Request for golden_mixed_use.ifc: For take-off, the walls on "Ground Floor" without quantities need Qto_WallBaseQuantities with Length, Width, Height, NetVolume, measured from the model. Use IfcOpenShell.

First a look at what the model holds.

```python
import ifcopenshell
import ifcopenshell.util.element
import ifcopenshell.util.unit

model = ifcopenshell.open("golden_mixed_use.ifc")
print(model.schema)
for unit_type in ("LENGTHUNIT", "AREAUNIT", "VOLUMEUNIT"):
    print(unit_type, ifcopenshell.util.unit.calculate_unit_scale(model, unit_type))
storey = next(s for s in model.by_type("IfcBuildingStorey") if s.Name == "Ground Floor")
walls = [e for e in ifcopenshell.util.element.get_decomposition(storey) if e.is_a("IfcWall")]
for e in sorted(walls, key=lambda e: e.id()):
    print(e.id(), e.is_a(), e.Name, list(ifcopenshell.util.element.get_psets(e, qtos_only=True)), sep=" | ")
```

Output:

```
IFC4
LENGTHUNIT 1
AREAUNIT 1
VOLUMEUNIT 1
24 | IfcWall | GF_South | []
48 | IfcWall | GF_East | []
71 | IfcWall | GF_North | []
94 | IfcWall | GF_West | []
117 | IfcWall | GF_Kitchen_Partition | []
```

```python
import ifcopenshell
import ifcopenshell.api.pset
import ifcopenshell.geom
import ifcopenshell.util.element
import ifcopenshell.util.shape
import ifcopenshell.util.unit

model = ifcopenshell.open("golden_mixed_use.ifc")
unit_scale = ifcopenshell.util.unit.calculate_unit_scale(model)
volume_scale = ifcopenshell.util.unit.calculate_unit_scale(model, "VOLUMEUNIT")
settings = ifcopenshell.geom.settings()

storey = next(s for s in model.by_type("IfcBuildingStorey") if s.Name == "Ground Floor")
walls = [e for e in ifcopenshell.util.element.get_decomposition(storey) if e.is_a("IfcWall")]

for e in sorted(walls, key=lambda e: e.id()):
    if ifcopenshell.util.element.get_psets(e, qtos_only=True, should_inherit=False):
        continue
    # Geometry comes back in metres, in the element's own axes.
    shape = ifcopenshell.geom.create_shape(settings, e)
    values = {
        "Length": ifcopenshell.util.shape.get_x(shape.geometry) / unit_scale,
        "Width": ifcopenshell.util.shape.get_y(shape.geometry) / unit_scale,
        "Height": ifcopenshell.util.shape.get_z(shape.geometry) / unit_scale,
        "NetVolume": ifcopenshell.util.shape.get_volume(shape.geometry) / volume_scale,
    }
    qto = ifcopenshell.api.pset.add_qto(model, product=e, name="Qto_WallBaseQuantities")
    ifcopenshell.api.pset.edit_qto(model, qto=qto, properties=values)
    print(e.id(), {k: round(v, 3) for k, v in values.items()})

model.write("golden_mixed_use_edited.ifc")
```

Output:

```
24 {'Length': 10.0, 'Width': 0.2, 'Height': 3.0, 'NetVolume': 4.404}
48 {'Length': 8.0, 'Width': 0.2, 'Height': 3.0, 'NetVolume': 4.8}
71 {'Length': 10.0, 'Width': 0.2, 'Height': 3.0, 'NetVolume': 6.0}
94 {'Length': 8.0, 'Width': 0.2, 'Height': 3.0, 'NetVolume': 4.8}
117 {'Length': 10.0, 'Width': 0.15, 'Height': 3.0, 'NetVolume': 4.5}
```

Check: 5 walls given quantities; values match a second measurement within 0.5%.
